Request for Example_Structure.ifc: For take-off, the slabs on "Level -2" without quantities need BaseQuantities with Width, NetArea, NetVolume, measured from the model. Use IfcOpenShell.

First a look at what the model holds.

```python
import ifcopenshell
import ifcopenshell.util.element
import ifcopenshell.util.unit

model = ifcopenshell.open("Example_Structure.ifc")
print(model.schema)
for unit_type in ("LENGTHUNIT", "AREAUNIT", "VOLUMEUNIT"):
    print(unit_type, ifcopenshell.util.unit.calculate_unit_scale(model, unit_type))
storey = next(s for s in model.by_type("IfcBuildingStorey") if s.Name == "Level -2")
slabs = [e for e in ifcopenshell.util.element.get_decomposition(storey) if e.is_a("IfcSlab")]
for e in sorted(slabs, key=lambda e: e.id()):
    print(e.id(), e.is_a(), e.Name, list(ifcopenshell.util.element.get_psets(e, qtos_only=True)), sep=" | ")
```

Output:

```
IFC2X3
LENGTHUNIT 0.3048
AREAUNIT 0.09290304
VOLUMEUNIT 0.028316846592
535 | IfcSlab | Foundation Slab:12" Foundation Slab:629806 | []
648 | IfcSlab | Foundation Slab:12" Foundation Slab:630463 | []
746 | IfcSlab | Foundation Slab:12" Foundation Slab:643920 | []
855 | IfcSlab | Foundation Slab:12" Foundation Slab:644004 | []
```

```python
import ifcopenshell
import ifcopenshell.api.pset
import ifcopenshell.geom
import ifcopenshell.util.element
import ifcopenshell.util.shape
import ifcopenshell.util.unit

model = ifcopenshell.open("Example_Structure.ifc")
unit_scale = ifcopenshell.util.unit.calculate_unit_scale(model)
area_scale = ifcopenshell.util.unit.calculate_unit_scale(model, "AREAUNIT")
volume_scale = ifcopenshell.util.unit.calculate_unit_scale(model, "VOLUMEUNIT")
settings = ifcopenshell.geom.settings()

storey = next(s for s in model.by_type("IfcBuildingStorey") if s.Name == "Level -2")
slabs = [e for e in ifcopenshell.util.element.get_decomposition(storey) if e.is_a("IfcSlab")]

for e in sorted(slabs, key=lambda e: e.id()):
    if ifcopenshell.util.element.get_psets(e, qtos_only=True, should_inherit=False):
        continue
    # Geometry comes back in metres, in the element's own axes.
    shape = ifcopenshell.geom.create_shape(settings, e)
    values = {
        "Width": ifcopenshell.util.shape.get_z(shape.geometry) / unit_scale,
        "NetArea": ifcopenshell.util.shape.get_footprint_area(shape.geometry) / area_scale,
        "NetVolume": ifcopenshell.util.shape.get_volume(shape.geometry) / volume_scale,
    }
    qto = ifcopenshell.api.pset.add_qto(model, product=e, name="BaseQuantities")
    ifcopenshell.api.pset.edit_qto(model, qto=qto, properties=values)
    print(e.id(), {k: round(v, 3) for k, v in values.items()})

model.write("Example_Structure_v2.ifc")
```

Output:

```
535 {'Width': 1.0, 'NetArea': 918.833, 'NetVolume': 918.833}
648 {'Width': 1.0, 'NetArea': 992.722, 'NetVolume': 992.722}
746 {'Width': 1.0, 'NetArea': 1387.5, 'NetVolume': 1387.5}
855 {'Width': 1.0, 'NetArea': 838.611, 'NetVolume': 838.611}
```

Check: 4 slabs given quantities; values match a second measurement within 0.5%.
